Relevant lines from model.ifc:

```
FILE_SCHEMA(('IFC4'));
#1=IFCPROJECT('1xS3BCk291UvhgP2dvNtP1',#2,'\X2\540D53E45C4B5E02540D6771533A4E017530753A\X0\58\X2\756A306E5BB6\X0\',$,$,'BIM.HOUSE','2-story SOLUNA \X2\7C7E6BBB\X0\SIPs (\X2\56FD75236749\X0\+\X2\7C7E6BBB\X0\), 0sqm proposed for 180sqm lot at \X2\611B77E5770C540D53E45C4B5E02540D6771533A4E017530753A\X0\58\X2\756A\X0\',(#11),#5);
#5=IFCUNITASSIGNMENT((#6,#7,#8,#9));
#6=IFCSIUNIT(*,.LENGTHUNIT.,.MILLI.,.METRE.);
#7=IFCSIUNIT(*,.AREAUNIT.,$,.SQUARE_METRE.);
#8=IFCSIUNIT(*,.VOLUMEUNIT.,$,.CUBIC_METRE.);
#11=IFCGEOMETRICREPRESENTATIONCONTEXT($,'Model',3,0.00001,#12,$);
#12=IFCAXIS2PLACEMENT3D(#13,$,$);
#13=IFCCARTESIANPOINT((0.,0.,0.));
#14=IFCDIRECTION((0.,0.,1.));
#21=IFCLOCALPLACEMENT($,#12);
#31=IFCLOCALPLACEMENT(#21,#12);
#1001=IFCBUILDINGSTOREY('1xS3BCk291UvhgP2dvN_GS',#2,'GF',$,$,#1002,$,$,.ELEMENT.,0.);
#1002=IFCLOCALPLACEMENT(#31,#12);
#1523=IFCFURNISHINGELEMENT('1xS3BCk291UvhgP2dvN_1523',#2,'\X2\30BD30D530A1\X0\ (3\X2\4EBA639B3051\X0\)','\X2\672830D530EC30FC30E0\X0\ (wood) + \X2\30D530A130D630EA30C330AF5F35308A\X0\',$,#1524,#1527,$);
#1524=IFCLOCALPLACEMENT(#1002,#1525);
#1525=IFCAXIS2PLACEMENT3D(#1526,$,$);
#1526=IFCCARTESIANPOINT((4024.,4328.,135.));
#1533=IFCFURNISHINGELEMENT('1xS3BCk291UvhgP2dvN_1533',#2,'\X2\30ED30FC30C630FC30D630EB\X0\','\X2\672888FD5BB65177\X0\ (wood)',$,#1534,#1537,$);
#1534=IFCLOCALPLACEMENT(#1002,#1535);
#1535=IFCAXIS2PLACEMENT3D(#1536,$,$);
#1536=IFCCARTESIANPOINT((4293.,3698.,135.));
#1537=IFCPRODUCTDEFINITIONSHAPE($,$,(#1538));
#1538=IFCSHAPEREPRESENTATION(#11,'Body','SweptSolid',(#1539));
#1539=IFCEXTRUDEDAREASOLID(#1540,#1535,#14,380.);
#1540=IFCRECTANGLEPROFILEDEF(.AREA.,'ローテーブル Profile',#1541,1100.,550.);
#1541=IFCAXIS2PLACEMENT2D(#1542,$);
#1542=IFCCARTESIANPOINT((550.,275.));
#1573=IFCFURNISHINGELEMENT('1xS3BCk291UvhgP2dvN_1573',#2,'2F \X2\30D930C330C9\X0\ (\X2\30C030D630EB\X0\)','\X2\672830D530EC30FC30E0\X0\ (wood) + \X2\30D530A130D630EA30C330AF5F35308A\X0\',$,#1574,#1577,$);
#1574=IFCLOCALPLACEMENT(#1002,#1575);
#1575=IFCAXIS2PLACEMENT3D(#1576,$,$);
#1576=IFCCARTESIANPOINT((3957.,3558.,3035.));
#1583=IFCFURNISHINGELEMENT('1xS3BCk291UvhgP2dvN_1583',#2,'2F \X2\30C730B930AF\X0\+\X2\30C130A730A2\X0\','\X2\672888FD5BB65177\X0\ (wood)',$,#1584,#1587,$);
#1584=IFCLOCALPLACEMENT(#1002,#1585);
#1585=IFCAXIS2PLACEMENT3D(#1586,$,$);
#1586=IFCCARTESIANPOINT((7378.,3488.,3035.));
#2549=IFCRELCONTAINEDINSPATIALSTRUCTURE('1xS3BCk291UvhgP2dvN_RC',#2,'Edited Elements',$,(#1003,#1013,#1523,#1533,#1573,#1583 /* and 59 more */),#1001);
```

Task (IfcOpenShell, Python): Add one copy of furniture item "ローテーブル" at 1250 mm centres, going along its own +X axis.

```python
import ifcopenshell
import ifcopenshell.api.geometry
import ifcopenshell.api.root
import ifcopenshell.util.element
import ifcopenshell.util.placement
import ifcopenshell.util.unit

model = ifcopenshell.open("model.ifc")
unit_scale = ifcopenshell.util.unit.calculate_unit_scale(model)


def reuse_history(source, copy):
    """copy_class also copies each property set's owner history, people and application; keep the originals."""
    for rel in copy.IsDefinedBy:
        if rel.is_a("IfcRelDefinesByProperties") and (history := rel.RelatingPropertyDefinition.OwnerHistory):
            rel.RelatingPropertyDefinition.OwnerHistory = source.OwnerHistory
            ifcopenshell.util.element.remove_deep2(model, history)


source = model.by_guid("1xS3BCk291UvhgP2dvN_1533")
base = ifcopenshell.util.placement.get_local_placement(source.ObjectPlacement)
step = base[:3, 0] * 1.25 / unit_scale

for i in range(1, 2):
    copy = ifcopenshell.api.root.copy_class(model, product=source)
    copy.Representation = ifcopenshell.util.element.copy_deep(
        model, source.Representation, exclude=["IfcGeometricRepresentationContext", "IfcRepresentationMap"]
    )
    reuse_history(source, copy)
    matrix = base.copy()
    matrix[:3, 3] += i * step
    print("added at", matrix[:3, 3].round(3) + 0.0)
    ifcopenshell.api.geometry.edit_object_placement(model, product=copy, matrix=matrix, is_si=False)

model.write("model_v2.ifc")
```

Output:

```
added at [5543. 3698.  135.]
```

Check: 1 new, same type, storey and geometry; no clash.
